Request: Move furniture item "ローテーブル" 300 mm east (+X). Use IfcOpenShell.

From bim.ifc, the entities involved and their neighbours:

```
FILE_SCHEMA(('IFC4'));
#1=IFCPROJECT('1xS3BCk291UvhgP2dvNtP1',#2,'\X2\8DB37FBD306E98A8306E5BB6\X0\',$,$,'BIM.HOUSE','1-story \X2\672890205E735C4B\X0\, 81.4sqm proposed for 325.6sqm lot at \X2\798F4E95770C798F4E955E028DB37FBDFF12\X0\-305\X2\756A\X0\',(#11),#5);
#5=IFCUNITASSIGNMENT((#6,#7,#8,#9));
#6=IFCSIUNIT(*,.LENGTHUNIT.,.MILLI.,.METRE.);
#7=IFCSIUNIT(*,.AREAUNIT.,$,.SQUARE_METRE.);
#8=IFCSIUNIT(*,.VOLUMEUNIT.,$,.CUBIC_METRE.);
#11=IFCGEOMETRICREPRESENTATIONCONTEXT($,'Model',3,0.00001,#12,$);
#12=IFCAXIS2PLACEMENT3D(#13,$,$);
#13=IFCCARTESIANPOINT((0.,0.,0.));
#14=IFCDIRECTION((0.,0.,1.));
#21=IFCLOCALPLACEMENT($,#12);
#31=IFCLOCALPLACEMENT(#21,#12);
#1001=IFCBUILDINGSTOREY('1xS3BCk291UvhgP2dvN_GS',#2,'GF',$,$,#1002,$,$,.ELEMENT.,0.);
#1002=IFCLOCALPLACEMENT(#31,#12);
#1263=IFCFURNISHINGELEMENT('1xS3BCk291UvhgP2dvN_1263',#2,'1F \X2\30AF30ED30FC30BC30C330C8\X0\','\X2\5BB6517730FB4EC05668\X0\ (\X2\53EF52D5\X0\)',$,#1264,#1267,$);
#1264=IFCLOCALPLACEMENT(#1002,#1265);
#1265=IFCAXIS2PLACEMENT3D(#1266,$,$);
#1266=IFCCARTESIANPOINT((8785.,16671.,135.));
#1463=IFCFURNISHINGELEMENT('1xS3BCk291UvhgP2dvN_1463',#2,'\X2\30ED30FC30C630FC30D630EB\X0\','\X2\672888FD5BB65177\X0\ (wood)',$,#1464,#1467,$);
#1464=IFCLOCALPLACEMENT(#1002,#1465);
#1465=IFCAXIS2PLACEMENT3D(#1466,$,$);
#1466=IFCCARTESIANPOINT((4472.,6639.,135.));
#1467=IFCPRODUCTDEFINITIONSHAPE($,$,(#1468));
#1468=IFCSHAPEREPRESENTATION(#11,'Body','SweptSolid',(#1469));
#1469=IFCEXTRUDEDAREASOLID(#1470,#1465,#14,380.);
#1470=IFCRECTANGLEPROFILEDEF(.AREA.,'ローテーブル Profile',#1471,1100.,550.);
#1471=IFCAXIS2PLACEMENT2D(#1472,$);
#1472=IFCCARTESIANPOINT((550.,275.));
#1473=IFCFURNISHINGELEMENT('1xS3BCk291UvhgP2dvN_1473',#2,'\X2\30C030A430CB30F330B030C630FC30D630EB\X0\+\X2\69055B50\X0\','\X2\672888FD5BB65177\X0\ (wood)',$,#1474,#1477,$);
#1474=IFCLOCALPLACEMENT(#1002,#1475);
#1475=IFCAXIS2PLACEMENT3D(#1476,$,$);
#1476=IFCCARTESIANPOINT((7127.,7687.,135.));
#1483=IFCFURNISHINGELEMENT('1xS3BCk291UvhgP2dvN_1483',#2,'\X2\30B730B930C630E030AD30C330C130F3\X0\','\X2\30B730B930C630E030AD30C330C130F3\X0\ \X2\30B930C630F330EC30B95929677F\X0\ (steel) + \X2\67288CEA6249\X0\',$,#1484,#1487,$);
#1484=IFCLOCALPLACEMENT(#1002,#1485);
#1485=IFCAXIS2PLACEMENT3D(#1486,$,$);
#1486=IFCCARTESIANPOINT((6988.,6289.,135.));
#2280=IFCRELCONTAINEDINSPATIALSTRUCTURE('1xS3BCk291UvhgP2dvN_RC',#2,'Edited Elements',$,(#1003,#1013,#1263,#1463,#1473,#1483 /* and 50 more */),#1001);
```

```python
import ifcopenshell
import ifcopenshell.api.geometry
import ifcopenshell.util.placement

model = ifcopenshell.open("bim.ifc")

item = model.by_guid("1xS3BCk291UvhgP2dvN_1463")
matrix = ifcopenshell.util.placement.get_local_placement(item.ObjectPlacement)
matrix[0, 3] += 300.0
ifcopenshell.api.geometry.edit_object_placement(model, product=item, matrix=matrix, is_si=False)

print(ifcopenshell.util.placement.get_local_placement(item.ObjectPlacement).round(3) + 0.0)

model.write("bim_v2.ifc")
```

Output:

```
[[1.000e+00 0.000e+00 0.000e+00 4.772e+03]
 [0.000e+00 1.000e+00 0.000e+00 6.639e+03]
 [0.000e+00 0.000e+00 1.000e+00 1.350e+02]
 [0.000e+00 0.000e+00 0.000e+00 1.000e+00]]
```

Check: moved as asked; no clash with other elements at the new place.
